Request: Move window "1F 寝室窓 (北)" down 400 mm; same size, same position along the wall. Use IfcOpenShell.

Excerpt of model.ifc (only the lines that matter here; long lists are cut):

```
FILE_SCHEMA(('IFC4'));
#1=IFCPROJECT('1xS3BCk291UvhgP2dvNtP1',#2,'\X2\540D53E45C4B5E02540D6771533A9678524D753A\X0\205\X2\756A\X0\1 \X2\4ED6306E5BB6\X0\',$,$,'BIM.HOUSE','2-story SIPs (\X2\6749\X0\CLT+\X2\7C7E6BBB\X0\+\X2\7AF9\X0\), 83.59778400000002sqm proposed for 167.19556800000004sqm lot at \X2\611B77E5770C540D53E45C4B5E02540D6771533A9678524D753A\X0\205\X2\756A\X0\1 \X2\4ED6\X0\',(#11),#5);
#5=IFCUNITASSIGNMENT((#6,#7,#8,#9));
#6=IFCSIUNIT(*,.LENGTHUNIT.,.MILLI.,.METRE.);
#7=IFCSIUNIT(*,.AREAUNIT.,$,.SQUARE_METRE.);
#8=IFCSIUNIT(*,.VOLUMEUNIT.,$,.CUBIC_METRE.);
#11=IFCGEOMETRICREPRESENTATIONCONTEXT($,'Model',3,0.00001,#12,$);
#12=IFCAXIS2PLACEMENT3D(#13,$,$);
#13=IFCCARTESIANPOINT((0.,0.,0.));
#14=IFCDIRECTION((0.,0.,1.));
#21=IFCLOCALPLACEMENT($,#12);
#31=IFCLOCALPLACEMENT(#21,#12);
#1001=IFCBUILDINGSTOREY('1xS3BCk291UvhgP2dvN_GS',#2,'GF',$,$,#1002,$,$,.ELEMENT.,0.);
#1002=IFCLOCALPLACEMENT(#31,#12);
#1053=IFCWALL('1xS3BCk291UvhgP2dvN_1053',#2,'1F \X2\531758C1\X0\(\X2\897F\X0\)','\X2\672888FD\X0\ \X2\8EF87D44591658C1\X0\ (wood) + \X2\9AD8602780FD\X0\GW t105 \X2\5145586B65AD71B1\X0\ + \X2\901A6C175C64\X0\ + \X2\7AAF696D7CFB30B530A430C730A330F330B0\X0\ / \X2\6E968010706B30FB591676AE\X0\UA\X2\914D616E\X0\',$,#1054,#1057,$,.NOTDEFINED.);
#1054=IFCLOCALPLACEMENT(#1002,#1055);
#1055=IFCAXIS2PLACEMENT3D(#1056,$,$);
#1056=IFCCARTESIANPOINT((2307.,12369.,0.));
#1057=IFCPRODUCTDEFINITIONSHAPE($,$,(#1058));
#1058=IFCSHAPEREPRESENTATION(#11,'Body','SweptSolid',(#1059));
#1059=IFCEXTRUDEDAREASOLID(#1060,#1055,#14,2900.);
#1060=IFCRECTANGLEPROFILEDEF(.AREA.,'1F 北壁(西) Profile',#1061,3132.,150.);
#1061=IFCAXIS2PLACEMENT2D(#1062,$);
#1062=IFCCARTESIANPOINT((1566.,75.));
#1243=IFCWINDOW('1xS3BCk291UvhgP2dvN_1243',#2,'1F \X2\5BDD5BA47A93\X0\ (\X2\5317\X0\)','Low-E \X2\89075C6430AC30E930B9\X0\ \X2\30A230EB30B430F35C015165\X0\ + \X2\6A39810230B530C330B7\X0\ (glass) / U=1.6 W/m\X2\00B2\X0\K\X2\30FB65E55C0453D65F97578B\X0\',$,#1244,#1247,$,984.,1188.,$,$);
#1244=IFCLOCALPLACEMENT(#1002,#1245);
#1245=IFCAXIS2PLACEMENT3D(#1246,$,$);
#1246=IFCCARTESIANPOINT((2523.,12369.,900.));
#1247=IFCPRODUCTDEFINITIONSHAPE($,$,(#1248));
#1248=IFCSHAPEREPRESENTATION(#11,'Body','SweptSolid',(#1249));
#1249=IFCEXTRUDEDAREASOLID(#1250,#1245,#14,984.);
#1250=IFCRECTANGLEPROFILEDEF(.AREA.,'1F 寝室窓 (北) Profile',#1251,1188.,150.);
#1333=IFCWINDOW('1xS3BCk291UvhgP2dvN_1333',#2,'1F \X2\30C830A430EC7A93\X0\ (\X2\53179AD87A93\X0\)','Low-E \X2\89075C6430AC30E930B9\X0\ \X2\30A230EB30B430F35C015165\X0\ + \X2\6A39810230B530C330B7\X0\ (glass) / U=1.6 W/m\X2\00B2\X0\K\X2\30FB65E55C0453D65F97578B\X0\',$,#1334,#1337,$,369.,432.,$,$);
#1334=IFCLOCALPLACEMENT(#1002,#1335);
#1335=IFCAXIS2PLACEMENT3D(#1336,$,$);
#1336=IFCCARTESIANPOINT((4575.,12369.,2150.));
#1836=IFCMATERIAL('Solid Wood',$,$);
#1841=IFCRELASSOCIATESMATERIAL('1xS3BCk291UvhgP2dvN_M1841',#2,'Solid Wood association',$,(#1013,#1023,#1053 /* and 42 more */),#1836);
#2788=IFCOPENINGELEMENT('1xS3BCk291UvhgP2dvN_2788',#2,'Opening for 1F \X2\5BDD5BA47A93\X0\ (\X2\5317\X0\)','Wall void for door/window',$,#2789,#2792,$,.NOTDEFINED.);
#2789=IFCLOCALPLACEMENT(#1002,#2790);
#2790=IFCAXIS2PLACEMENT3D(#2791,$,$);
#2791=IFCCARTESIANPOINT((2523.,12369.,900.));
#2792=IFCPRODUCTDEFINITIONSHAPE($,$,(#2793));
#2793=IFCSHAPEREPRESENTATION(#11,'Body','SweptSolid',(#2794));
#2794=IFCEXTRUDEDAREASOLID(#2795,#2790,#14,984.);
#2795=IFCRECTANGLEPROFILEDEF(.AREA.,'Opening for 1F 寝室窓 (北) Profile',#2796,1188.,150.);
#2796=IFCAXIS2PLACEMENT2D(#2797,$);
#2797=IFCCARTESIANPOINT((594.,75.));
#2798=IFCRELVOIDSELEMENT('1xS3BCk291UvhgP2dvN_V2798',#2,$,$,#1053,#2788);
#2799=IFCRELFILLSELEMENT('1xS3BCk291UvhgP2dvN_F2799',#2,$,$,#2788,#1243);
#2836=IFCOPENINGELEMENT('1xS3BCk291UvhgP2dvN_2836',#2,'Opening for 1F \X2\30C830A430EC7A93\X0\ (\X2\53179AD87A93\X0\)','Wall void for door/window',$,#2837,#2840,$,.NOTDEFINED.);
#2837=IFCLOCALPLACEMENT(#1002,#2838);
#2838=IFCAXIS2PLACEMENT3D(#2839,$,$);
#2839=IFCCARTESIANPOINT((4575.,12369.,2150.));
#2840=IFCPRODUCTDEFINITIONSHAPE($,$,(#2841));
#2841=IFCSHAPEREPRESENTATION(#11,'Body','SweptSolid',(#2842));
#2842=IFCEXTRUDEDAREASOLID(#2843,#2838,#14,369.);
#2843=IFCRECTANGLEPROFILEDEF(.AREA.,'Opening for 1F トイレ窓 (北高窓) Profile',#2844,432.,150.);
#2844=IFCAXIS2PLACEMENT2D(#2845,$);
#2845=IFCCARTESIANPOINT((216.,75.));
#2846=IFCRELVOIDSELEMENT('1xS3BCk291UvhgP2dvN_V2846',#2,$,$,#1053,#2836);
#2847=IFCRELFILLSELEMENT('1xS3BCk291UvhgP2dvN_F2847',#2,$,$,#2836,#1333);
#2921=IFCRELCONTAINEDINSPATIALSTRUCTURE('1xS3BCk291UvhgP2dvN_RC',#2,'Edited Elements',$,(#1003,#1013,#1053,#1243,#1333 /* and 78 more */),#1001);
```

```python
import numpy as np
import ifcopenshell
import ifcopenshell.api.geometry
import ifcopenshell.util.placement
import ifcopenshell.util.unit

model = ifcopenshell.open("model.ifc")
unit_scale = ifcopenshell.util.unit.calculate_unit_scale(model)

window = model.by_guid("1xS3BCk291UvhgP2dvN_1243")
opening = window.FillsVoids[0].RelatingOpeningElement
dz = -0.4 / unit_scale

shift = np.array([0.0, 0.0, dz])
# The window is not placed relative to its opening, so move both.
for product in (opening, window):
    matrix = ifcopenshell.util.placement.get_local_placement(product.ObjectPlacement)
    matrix[:3, 3] += shift
    ifcopenshell.api.geometry.edit_object_placement(model, product=product, matrix=matrix, is_si=False)

print(f"moved by {dz * unit_scale:+.3f} m")

model.write("model_rev.ifc")
```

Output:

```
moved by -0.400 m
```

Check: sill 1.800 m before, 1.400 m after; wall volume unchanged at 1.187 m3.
